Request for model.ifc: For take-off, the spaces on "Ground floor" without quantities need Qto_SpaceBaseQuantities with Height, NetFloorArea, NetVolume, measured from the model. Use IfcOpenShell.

First a look at what the model holds.

```python
import ifcopenshell
import ifcopenshell.util.element
import ifcopenshell.util.unit

model = ifcopenshell.open("model.ifc")
print(model.schema)
for unit_type in ("LENGTHUNIT", "AREAUNIT", "VOLUMEUNIT"):
    print(unit_type, ifcopenshell.util.unit.calculate_unit_scale(model, unit_type))
storey = next(s for s in model.by_type("IfcBuildingStorey") if s.Name == "Ground floor")
spaces = [e for e in ifcopenshell.util.element.get_decomposition(storey) if e.is_a("IfcSpace")]
for e in sorted(spaces, key=lambda e: e.id()):
    print(e.id(), e.is_a(), e.Name, list(ifcopenshell.util.element.get_psets(e, qtos_only=True)), sep=" | ")
```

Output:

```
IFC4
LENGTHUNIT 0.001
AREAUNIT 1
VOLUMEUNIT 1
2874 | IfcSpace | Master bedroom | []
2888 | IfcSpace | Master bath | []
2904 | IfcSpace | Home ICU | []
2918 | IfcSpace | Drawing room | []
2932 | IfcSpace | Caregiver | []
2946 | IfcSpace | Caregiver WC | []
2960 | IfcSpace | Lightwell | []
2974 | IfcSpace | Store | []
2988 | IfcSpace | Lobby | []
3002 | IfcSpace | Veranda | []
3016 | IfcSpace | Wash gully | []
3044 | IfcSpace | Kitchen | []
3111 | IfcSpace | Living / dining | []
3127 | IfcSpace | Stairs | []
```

```python
import ifcopenshell
import ifcopenshell.api.pset
import ifcopenshell.geom
import ifcopenshell.util.element
import ifcopenshell.util.shape
import ifcopenshell.util.unit

model = ifcopenshell.open("model.ifc")
unit_scale = ifcopenshell.util.unit.calculate_unit_scale(model)
area_scale = ifcopenshell.util.unit.calculate_unit_scale(model, "AREAUNIT")
volume_scale = ifcopenshell.util.unit.calculate_unit_scale(model, "VOLUMEUNIT")
settings = ifcopenshell.geom.settings()

storey = next(s for s in model.by_type("IfcBuildingStorey") if s.Name == "Ground floor")
spaces = [e for e in ifcopenshell.util.element.get_decomposition(storey) if e.is_a("IfcSpace")]

for e in sorted(spaces, key=lambda e: e.id()):
    if ifcopenshell.util.element.get_psets(e, qtos_only=True, should_inherit=False):
        continue
    # Geometry comes back in metres, in the element's own axes.
    shape = ifcopenshell.geom.create_shape(settings, e)
    values = {
        "Height": ifcopenshell.util.shape.get_z(shape.geometry) / unit_scale,
        "NetFloorArea": ifcopenshell.util.shape.get_footprint_area(shape.geometry) / area_scale,
        "NetVolume": ifcopenshell.util.shape.get_volume(shape.geometry) / volume_scale,
    }
    qto = ifcopenshell.api.pset.add_qto(model, product=e, name="Qto_SpaceBaseQuantities")
    ifcopenshell.api.pset.edit_qto(model, qto=qto, properties=values)
    print(e.id(), {k: round(v, 3) for k, v in values.items()})

model.write("model_edited.ifc")
```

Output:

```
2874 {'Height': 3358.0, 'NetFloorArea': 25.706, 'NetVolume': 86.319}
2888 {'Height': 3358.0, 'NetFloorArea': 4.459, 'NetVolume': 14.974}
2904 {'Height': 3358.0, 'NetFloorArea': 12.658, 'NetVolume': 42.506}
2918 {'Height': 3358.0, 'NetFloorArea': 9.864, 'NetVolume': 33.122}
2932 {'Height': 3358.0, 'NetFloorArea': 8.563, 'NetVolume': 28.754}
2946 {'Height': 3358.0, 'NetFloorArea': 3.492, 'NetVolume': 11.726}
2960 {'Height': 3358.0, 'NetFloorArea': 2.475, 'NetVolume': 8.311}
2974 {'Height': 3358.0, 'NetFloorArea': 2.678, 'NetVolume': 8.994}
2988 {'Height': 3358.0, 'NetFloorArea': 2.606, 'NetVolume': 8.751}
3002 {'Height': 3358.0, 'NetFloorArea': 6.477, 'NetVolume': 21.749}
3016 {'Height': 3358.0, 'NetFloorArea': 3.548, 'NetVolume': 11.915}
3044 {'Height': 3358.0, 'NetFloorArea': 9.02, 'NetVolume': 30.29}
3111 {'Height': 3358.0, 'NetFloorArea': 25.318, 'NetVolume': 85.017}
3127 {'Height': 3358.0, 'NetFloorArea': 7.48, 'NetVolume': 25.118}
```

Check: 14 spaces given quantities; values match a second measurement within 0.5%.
